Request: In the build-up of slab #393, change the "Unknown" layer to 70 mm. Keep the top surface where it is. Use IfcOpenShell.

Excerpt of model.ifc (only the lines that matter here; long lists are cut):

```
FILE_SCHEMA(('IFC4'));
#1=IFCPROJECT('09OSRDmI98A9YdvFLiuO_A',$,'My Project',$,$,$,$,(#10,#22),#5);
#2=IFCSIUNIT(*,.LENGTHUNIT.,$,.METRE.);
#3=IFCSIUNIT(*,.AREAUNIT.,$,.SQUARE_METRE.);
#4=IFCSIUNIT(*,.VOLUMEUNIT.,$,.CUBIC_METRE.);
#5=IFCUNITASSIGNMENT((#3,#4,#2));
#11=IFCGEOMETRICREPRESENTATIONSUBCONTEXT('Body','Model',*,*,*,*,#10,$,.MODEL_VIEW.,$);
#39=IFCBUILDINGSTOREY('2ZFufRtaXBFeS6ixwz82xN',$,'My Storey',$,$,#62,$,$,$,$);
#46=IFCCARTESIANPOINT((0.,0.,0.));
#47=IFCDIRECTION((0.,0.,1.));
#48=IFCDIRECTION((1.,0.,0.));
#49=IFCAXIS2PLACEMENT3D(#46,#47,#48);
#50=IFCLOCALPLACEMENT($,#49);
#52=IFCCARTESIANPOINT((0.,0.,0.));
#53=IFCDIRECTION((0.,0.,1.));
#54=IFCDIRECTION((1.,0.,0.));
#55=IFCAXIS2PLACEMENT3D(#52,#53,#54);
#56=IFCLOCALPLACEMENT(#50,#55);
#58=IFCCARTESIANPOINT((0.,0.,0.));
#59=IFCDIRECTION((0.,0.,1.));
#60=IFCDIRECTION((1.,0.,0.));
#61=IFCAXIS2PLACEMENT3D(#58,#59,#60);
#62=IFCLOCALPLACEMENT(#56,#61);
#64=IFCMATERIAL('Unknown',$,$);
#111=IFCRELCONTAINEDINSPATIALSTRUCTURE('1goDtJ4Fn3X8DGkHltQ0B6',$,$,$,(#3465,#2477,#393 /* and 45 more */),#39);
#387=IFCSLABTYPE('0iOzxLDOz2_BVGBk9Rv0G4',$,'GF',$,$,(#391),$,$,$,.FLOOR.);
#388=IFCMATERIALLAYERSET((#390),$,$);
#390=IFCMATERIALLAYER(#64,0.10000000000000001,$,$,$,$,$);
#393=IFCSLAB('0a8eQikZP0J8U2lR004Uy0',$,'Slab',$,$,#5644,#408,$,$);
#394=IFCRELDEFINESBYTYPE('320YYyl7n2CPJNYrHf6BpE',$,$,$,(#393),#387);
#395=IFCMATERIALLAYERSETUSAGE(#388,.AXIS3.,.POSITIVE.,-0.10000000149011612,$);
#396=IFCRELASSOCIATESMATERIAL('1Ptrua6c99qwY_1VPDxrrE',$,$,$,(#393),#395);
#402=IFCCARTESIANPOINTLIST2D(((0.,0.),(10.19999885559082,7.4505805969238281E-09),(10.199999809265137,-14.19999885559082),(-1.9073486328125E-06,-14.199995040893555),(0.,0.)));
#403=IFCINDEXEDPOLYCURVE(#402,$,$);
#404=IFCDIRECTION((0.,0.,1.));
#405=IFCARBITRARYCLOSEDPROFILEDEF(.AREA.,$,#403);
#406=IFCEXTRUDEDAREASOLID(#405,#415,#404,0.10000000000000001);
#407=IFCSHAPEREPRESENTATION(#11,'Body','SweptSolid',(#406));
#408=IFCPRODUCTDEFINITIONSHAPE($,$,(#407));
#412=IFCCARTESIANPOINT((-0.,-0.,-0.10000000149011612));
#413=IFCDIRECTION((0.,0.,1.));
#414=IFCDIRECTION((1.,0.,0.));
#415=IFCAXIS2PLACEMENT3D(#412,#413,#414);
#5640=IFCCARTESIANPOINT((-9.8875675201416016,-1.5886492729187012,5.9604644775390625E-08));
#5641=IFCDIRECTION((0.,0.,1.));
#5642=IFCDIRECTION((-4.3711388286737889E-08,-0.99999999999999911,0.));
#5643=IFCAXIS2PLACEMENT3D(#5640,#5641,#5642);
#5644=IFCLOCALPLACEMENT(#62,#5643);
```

```python
import ifcopenshell
import ifcopenshell.util.element
import ifcopenshell.util.representation
import ifcopenshell.util.unit

model = ifcopenshell.open("model.ifc")
unit_scale = ifcopenshell.util.unit.calculate_unit_scale(model)

layer_set = model.by_id(388)
layer = next(l for l in layer_set.MaterialLayers if l.Material and l.Material.Name == "Unknown")
change = 0.07 / unit_scale - layer.LayerThickness
layer.LayerThickness += change

# Geometry does not follow the layer set by itself.
slabs = [e for e in ifcopenshell.util.element.get_elements_by_material(model, layer_set) if e.is_a("IfcSlab")]
for slab in sorted(slabs, key=lambda e: e.id()):
    body = ifcopenshell.util.representation.get_representation(slab, "Model", "Body")
    solid = body.Items[0]
    old_depth = solid.Depth
    solid.Depth += change
    # Extruded upwards: lower the start of the extrusion so the top stays.
    x, y, z = solid.Position.Location.Coordinates
    solid.Position.Location = model.createIfcCartesianPoint((x, y, z - change))
    print(slab.id(), f"{old_depth:g} -> {solid.Depth:g}")

# The layers are counted up from the underside, which has moved.
for usage in {ifcopenshell.util.element.get_material(slab) for slab in slabs}:
    usage.OffsetFromReferenceLine -= change

model.write("model_updated.ifc")
```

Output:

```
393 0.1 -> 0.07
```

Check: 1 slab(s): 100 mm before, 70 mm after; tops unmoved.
